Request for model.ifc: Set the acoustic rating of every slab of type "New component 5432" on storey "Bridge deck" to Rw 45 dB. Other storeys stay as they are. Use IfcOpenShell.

First a look at what the model holds.

```python
import ifcopenshell
import ifcopenshell.util.element

model = ifcopenshell.open("model.ifc")
print(model.schema)
storey = next(s for s in model.by_type("IfcBuildingStorey") if s.Name == "Bridge deck")
slabs = [e for e in ifcopenshell.util.element.get_decomposition(storey) if e.is_a("IfcSlab")]
seen = {}
for e in slabs:
    element_type = ifcopenshell.util.element.get_type(e)
    key = (element_type.Name if element_type != e and element_type else None, ifcopenshell.util.element.get_pset(e, "Pset_SlabCommon", "AcousticRating"))
    seen[key] = seen.get(key, 0) + 1
for (name, value), count in sorted(seen.items(), key=str):
    print(count, "x", name, "|", value)
```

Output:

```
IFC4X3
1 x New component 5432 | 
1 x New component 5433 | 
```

```python
import ifcopenshell
import ifcopenshell.api.pset
import ifcopenshell.util.element

model = ifcopenshell.open("model.ifc")

storey = next(s for s in model.by_type("IfcBuildingStorey") if s.Name == "Bridge deck")
slabs = [e for e in ifcopenshell.util.element.get_decomposition(storey) if e.is_a("IfcSlab")]

count = 0
for e in slabs:
    element_type = ifcopenshell.util.element.get_type(e)
    if element_type in (None, e) or element_type.Name != "New component 5432":
        continue
    # add_pset returns the element's existing set when there is one.
    pset = ifcopenshell.api.pset.add_pset(model, product=e, name="Pset_SlabCommon")
    ifcopenshell.api.pset.edit_pset(model, pset=pset, properties={"AcousticRating": "Rw 45 dB"})
    count += 1

print(count, "slabs updated")

model.write("model_rev.ifc")
```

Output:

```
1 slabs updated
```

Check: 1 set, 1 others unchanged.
